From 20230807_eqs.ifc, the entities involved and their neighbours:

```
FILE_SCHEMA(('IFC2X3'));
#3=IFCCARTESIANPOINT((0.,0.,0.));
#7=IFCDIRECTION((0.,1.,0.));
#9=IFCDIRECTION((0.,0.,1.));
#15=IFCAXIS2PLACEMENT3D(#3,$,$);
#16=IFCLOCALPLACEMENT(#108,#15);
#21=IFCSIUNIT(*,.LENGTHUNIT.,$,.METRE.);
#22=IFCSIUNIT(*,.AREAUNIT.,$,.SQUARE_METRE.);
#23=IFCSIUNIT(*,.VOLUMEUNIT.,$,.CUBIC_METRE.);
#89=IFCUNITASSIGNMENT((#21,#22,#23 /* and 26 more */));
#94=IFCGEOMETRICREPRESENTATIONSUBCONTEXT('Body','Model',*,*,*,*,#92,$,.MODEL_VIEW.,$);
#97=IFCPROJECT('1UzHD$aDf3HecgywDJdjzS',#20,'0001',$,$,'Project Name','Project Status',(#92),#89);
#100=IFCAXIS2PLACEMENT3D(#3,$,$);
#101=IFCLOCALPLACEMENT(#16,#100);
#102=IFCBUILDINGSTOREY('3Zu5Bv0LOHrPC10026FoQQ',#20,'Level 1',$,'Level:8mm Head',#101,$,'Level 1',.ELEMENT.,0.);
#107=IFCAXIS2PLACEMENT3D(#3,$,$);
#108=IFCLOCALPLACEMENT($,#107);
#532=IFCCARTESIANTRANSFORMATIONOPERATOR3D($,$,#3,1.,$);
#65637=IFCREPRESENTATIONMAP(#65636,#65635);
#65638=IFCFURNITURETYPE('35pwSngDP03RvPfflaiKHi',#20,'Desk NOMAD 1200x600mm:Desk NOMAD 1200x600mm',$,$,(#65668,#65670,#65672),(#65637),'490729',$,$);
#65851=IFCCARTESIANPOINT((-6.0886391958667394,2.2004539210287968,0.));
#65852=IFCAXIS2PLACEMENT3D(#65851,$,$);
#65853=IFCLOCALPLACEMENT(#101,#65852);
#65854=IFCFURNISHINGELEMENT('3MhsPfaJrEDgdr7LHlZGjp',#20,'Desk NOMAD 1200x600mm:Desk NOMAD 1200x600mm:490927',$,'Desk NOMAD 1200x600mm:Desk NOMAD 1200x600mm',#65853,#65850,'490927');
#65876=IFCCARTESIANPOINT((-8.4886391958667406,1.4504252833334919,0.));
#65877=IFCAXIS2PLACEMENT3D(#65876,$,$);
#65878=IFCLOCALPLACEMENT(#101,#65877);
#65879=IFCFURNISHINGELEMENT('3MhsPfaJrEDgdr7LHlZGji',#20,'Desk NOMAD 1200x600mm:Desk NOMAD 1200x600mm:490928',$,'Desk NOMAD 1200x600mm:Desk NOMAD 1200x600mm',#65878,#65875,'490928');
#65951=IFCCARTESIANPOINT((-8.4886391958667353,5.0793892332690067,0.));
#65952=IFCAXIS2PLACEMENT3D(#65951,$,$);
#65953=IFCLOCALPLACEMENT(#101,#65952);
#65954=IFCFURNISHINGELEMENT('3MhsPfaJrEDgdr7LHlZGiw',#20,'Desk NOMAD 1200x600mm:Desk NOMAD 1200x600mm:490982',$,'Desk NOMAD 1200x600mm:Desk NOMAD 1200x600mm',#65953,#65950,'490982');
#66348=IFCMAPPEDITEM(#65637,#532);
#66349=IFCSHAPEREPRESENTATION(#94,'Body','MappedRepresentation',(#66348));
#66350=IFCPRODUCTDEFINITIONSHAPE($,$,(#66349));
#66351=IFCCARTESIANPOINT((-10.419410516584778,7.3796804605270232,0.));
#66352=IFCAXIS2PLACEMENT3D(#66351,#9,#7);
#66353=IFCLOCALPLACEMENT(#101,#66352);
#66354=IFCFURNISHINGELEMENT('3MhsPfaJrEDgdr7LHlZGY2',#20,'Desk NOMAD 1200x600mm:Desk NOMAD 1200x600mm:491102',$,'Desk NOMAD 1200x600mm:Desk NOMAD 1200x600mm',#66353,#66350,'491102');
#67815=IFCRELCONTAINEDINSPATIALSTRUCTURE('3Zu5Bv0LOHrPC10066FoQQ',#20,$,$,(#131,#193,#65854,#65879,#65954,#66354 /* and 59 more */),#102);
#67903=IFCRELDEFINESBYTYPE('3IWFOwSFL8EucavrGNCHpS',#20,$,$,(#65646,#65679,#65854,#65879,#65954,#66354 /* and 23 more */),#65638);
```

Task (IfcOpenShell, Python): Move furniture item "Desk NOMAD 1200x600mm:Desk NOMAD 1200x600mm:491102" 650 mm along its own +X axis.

```python
import ifcopenshell
import ifcopenshell.api.geometry
import ifcopenshell.util.placement
import ifcopenshell.util.unit

model = ifcopenshell.open("20230807_eqs.ifc")
unit_scale = ifcopenshell.util.unit.calculate_unit_scale(model)

item = model.by_guid("3MhsPfaJrEDgdr7LHlZGY2")
matrix = ifcopenshell.util.placement.get_local_placement(item.ObjectPlacement)
matrix[:3, 3] += matrix[:3, 0] * 0.65 / unit_scale
ifcopenshell.api.geometry.edit_object_placement(model, product=item, matrix=matrix, is_si=False)

print(ifcopenshell.util.placement.get_local_placement(item.ObjectPlacement).round(3) + 0.0)

model.write("20230807_eqs-out.ifc")
```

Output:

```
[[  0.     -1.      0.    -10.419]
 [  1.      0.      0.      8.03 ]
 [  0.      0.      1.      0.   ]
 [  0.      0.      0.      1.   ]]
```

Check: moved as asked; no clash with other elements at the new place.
